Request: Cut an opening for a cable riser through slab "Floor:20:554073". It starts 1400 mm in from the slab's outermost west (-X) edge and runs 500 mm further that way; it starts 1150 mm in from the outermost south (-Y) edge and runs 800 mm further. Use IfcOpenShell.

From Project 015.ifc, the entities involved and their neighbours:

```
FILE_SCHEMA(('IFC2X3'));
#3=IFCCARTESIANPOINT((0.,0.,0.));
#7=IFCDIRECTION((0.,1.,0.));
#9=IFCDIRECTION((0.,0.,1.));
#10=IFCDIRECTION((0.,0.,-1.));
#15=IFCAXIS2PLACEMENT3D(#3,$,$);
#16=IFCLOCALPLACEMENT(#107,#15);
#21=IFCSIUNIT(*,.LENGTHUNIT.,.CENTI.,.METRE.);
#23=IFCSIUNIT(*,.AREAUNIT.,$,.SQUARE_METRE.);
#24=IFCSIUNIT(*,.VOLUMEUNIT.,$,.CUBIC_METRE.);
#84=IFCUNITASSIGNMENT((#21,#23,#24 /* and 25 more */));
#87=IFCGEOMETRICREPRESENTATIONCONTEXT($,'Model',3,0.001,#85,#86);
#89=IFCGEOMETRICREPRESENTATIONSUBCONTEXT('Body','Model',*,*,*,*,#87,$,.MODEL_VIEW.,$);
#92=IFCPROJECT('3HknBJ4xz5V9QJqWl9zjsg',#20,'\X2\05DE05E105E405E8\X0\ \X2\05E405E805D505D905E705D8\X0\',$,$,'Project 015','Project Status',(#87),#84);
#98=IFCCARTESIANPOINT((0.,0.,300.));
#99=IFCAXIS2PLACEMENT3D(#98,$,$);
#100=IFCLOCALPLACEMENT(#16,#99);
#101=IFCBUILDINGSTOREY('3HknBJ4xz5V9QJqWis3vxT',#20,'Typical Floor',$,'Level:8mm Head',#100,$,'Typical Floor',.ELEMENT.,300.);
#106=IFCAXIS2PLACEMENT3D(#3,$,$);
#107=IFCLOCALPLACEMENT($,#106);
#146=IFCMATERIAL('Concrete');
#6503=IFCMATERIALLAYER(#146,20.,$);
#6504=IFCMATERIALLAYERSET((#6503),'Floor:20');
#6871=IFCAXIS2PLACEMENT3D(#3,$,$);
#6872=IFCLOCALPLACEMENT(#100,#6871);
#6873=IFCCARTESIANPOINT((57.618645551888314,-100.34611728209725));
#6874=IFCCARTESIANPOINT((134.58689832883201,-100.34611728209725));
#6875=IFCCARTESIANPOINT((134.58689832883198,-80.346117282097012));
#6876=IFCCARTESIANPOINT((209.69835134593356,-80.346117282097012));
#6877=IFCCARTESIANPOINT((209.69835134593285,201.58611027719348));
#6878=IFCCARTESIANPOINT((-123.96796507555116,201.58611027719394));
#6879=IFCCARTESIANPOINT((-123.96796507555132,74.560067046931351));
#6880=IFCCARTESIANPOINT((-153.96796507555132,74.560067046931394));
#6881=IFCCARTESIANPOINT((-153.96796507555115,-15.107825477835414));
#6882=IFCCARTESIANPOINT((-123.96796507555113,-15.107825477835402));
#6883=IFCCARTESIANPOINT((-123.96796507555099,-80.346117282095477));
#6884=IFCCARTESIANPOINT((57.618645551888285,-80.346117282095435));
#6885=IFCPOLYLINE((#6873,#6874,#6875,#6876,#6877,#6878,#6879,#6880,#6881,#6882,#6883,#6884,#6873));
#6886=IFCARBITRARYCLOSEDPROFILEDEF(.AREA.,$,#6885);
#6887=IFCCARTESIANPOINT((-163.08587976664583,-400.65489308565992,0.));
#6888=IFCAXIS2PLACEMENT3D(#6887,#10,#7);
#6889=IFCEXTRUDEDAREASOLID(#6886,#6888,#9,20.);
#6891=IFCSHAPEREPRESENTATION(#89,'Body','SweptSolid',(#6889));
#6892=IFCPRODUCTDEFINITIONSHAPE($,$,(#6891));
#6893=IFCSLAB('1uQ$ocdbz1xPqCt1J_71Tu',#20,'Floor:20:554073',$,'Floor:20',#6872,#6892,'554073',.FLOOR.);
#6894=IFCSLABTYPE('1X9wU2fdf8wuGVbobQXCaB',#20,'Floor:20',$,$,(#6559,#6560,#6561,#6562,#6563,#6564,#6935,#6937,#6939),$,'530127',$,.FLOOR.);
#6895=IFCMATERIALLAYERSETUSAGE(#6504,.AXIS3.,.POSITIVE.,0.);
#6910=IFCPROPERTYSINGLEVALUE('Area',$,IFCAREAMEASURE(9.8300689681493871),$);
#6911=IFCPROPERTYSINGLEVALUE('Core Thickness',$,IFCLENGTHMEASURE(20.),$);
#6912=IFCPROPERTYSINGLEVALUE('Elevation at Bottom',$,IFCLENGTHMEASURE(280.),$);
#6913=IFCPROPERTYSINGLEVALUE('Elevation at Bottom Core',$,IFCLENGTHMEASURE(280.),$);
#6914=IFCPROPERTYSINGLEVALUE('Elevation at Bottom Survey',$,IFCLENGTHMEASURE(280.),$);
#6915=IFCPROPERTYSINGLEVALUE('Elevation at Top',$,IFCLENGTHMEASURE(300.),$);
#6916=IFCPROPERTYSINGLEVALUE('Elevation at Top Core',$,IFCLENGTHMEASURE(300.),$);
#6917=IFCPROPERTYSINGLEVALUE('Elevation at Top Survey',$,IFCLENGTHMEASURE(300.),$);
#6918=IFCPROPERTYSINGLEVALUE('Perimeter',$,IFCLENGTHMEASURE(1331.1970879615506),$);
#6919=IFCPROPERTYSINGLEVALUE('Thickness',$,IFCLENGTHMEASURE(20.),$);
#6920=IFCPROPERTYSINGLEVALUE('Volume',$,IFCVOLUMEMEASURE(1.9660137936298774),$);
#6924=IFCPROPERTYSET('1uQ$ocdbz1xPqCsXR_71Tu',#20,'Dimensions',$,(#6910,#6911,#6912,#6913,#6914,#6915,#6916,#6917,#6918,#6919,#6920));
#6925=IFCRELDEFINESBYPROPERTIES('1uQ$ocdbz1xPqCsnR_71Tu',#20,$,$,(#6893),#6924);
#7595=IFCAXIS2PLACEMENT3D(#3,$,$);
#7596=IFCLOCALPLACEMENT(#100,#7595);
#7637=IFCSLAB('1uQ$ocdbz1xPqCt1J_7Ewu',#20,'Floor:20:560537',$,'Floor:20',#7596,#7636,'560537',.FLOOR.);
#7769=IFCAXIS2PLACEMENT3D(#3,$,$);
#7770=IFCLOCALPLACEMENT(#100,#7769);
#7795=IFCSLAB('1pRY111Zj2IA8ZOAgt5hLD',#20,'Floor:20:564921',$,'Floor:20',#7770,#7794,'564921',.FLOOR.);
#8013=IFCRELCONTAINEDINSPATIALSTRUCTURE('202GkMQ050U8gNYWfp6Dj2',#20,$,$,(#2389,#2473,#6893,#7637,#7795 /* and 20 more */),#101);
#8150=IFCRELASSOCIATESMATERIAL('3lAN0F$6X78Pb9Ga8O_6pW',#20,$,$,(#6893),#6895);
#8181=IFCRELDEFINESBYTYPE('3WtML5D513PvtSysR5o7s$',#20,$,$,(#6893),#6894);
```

```python
import numpy as np
import ifcopenshell
import ifcopenshell.api.feature
import ifcopenshell.api.geometry
import ifcopenshell.api.pset
import ifcopenshell.api.root
import ifcopenshell.geom
import ifcopenshell.util.element
import ifcopenshell.util.placement
import ifcopenshell.util.representation
import ifcopenshell.util.shape
import ifcopenshell.util.unit

model = ifcopenshell.open("Project 015.ifc")
unit_scale = ifcopenshell.util.unit.calculate_unit_scale(model)
area_scale = ifcopenshell.util.unit.calculate_unit_scale(model, "AREAUNIT")
volume_scale = ifcopenshell.util.unit.calculate_unit_scale(model, "VOLUMEUNIT")
settings = ifcopenshell.geom.settings()


def volume(element):
    """Net volume in cubic metres, openings subtracted."""
    shape = ifcopenshell.geom.create_shape(settings, element)
    return ifcopenshell.util.shape.get_volume(shape.geometry)


slab = model.by_guid("1uQ$ocdbz1xPqCt1J_71Tu")
before = volume(slab)

# Extent in the slab's own axes, in metres. The edges named are its -X and -Y sides.
slab_shape = ifcopenshell.geom.create_shape(settings, slab)
vertices = ifcopenshell.util.shape.get_vertices(slab_shape.geometry)
x_min, y_min, bottom = vertices.min(axis=0)
top = vertices[:, 2].max()

opening = ifcopenshell.api.root.create_entity(model, ifc_class="IfcOpeningElement", name="Cable riser opening")
context = ifcopenshell.util.representation.get_context(model, "Model", "Body", "MODEL_VIEW")
width, depth = 0.5, 0.8
outline = [(0.0, 0.0), (width, 0.0), (width, depth), (0.0, depth), (0.0, 0.0)]
# Overshoot both faces by 50 mm so the cut is clean.
shape = ifcopenshell.api.geometry.add_slab_representation(
    model, context=context, depth=top - bottom + 0.1, polyline=outline
)
ifcopenshell.api.geometry.assign_representation(model, product=opening, representation=shape)

matrix = ifcopenshell.util.placement.get_local_placement(slab.ObjectPlacement)
matrix[:, 3] = matrix @ np.append(np.array([x_min + 1.4, y_min + 1.15, bottom - 0.05]) / unit_scale, 1.0)
ifcopenshell.api.geometry.edit_object_placement(model, product=opening, matrix=matrix, is_si=False)
ifcopenshell.api.feature.add_feature(model, feature=opening, element=slab)

after = volume(slab)

# Update the slab's stored quantities.
pset = model.by_id(ifcopenshell.util.element.get_pset(slab, "Dimensions", should_inherit=False)["id"])
ifcopenshell.api.pset.edit_pset(model, pset=pset, properties={
    "Area": model.create_entity("IfcAreaMeasure", after / (top - bottom) / area_scale),
    "Volume": model.create_entity("IfcVolumeMeasure", after / volume_scale),
})

print(f"slab volume {before:.3f} -> {after:.3f} m3")

model.write("Project 015-out.ifc")
```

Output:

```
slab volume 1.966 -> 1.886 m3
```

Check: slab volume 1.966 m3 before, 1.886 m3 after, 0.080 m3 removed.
